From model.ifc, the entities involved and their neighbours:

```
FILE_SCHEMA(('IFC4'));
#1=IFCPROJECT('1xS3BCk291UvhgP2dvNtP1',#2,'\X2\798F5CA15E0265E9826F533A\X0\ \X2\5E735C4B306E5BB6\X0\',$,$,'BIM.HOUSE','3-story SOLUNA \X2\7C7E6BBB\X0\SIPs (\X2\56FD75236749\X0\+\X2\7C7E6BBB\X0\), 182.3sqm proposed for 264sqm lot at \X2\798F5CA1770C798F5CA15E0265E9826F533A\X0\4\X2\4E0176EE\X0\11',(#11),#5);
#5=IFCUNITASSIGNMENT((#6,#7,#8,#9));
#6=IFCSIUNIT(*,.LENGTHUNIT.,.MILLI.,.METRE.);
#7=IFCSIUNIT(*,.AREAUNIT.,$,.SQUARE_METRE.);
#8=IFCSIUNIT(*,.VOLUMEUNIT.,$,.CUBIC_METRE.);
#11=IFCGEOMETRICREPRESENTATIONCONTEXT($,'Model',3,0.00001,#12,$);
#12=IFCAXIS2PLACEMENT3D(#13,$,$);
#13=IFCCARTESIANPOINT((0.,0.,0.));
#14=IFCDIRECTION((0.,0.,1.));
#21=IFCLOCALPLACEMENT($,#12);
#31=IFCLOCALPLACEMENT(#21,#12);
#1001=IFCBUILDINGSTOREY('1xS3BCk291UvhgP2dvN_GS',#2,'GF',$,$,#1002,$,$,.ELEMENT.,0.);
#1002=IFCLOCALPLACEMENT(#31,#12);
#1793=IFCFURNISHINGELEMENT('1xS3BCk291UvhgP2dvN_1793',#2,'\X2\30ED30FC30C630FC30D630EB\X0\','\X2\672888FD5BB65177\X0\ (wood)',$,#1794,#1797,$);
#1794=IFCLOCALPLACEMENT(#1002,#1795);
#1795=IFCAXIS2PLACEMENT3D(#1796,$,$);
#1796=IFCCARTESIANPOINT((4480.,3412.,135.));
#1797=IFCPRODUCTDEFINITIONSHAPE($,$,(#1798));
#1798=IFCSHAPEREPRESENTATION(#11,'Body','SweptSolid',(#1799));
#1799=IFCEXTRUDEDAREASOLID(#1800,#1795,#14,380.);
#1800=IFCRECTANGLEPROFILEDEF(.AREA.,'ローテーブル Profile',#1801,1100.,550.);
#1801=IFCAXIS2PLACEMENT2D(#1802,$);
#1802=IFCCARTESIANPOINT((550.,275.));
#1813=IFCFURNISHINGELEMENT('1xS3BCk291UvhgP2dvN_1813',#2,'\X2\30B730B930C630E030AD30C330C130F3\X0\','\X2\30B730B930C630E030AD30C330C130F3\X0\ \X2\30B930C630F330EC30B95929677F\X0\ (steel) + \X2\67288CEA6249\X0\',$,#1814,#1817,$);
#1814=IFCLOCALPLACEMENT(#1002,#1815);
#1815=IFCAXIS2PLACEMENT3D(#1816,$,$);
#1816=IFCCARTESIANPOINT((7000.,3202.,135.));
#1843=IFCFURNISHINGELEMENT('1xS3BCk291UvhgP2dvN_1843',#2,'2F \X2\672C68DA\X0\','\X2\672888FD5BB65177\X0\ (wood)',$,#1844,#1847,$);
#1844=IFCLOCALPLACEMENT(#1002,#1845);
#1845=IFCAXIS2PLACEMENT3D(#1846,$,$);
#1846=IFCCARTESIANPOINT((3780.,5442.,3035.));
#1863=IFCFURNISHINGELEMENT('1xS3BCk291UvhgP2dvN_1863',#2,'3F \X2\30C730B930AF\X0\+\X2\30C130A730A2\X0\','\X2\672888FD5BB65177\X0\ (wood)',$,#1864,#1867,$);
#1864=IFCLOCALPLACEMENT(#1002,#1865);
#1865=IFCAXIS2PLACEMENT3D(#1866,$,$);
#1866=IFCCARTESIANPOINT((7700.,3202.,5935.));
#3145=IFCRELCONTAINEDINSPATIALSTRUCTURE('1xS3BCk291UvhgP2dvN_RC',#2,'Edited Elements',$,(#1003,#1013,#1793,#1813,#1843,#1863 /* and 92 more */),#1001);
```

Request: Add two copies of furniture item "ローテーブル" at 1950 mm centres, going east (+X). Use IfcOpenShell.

```python
import numpy as np
import ifcopenshell
import ifcopenshell.api.geometry
import ifcopenshell.api.root
import ifcopenshell.util.element
import ifcopenshell.util.placement

model = ifcopenshell.open("model.ifc")


def reuse_history(source, copy):
    """copy_class also copies each property set's owner history, people and application; keep the originals."""
    for rel in copy.IsDefinedBy:
        if rel.is_a("IfcRelDefinesByProperties") and (history := rel.RelatingPropertyDefinition.OwnerHistory):
            rel.RelatingPropertyDefinition.OwnerHistory = source.OwnerHistory
            ifcopenshell.util.element.remove_deep2(model, history)


source = model.by_id(1793)
base = ifcopenshell.util.placement.get_local_placement(source.ObjectPlacement)
step = np.array([1.0, 0.0, 0.0]) * 1950.0

for i in range(1, 3):
    copy = ifcopenshell.api.root.copy_class(model, product=source)
    copy.Representation = ifcopenshell.util.element.copy_deep(
        model, source.Representation, exclude=["IfcGeometricRepresentationContext", "IfcRepresentationMap"]
    )
    reuse_history(source, copy)
    matrix = base.copy()
    matrix[:3, 3] += i * step
    print("added at", matrix[:3, 3].round(3) + 0.0)
    ifcopenshell.api.geometry.edit_object_placement(model, product=copy, matrix=matrix, is_si=False)

model.write("model_v2.ifc")
```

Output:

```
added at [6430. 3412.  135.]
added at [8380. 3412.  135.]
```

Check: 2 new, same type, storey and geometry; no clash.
